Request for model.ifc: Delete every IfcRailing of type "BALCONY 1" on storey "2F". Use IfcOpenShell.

First a look at what the model holds.

```python
import ifcopenshell
import ifcopenshell.util.element

model = ifcopenshell.open("model.ifc")
print(model.schema)
storey = next(s for s in model.by_type("IfcBuildingStorey") if s.Name == "2F")
railings = [e for e in ifcopenshell.util.element.get_decomposition(storey) if e.is_a("IfcRailing")]
seen = {}
for e in railings:
    element_type = ifcopenshell.util.element.get_type(e)
    name = element_type.Name if element_type not in (None, e) else None
    seen[name] = seen.get(name, 0) + 1
for name, count in sorted(seen.items(), key=str):
    print(count, "x", name)
```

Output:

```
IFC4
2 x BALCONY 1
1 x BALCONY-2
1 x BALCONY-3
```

```python
import ifcopenshell
import ifcopenshell.api.root
import ifcopenshell.util.element

model = ifcopenshell.open("model.ifc")

storey = next(s for s in model.by_type("IfcBuildingStorey") if s.Name == "2F")
railings = [e for e in ifcopenshell.util.element.get_decomposition(storey) if e.is_a("IfcRailing")]
targets = [e for e in railings if (t := ifcopenshell.util.element.get_type(e)) not in (None, e) and t.Name == "BALCONY 1"]

for e in targets:
    ifcopenshell.api.root.remove_product(model, product=e)
print(len(targets), "removed")

model.write("model-out.ifc")
```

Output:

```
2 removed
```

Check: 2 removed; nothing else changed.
